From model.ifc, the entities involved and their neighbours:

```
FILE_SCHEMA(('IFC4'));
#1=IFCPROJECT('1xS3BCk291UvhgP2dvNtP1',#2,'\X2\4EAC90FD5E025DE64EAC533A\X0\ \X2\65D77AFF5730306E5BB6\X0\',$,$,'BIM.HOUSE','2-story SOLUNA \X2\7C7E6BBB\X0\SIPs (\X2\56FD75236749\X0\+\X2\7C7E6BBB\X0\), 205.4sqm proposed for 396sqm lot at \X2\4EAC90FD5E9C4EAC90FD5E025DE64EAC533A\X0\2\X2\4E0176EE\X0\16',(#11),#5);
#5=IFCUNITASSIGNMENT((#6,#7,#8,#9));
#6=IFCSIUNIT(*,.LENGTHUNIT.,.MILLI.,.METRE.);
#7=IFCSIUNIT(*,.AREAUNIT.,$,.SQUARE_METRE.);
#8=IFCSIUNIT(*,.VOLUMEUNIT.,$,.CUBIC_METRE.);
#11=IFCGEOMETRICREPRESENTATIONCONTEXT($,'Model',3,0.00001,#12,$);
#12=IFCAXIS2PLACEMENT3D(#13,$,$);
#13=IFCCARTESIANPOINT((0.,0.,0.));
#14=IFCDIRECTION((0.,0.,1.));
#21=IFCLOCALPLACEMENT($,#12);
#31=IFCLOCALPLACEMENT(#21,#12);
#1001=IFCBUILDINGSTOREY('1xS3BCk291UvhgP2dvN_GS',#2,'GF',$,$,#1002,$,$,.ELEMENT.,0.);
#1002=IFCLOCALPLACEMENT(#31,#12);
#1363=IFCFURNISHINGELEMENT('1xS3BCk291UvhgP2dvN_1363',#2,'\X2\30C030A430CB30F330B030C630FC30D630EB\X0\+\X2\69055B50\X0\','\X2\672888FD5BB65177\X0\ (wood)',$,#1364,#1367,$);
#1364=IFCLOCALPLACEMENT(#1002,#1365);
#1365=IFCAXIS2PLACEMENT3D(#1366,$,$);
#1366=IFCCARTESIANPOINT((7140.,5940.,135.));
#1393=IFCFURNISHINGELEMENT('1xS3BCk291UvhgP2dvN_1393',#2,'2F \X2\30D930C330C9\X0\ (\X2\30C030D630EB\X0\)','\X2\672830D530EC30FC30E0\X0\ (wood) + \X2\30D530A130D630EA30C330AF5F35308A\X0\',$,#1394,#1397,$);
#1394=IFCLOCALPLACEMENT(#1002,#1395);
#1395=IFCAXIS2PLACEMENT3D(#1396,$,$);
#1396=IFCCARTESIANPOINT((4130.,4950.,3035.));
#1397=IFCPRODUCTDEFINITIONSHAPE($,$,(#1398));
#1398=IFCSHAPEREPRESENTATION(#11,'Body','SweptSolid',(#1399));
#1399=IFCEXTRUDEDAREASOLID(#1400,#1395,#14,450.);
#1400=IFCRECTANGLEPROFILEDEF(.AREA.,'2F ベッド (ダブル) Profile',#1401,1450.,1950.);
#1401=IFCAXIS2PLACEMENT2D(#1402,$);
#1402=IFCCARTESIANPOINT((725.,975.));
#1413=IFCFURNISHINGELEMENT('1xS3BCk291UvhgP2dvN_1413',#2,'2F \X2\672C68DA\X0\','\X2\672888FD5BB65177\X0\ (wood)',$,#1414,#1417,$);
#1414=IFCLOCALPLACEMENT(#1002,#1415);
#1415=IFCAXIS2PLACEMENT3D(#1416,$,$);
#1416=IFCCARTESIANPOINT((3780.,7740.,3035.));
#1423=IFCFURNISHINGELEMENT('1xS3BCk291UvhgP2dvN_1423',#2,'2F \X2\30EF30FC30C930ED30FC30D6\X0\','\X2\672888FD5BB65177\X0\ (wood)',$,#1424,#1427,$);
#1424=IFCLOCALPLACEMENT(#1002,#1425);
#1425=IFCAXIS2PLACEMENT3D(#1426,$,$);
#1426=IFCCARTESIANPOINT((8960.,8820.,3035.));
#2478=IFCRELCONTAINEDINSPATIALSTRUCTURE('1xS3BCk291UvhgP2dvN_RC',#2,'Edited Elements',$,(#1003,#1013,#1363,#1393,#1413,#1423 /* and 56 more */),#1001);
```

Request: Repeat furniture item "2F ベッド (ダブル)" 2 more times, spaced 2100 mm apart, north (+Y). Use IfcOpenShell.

```python
import numpy as np
import ifcopenshell
import ifcopenshell.api.geometry
import ifcopenshell.api.root
import ifcopenshell.util.element
import ifcopenshell.util.placement

model = ifcopenshell.open("model.ifc")


def reuse_history(source, copy):
    """copy_class also copies each property set's owner history, people and application; keep the originals."""
    for rel in copy.IsDefinedBy:
        if rel.is_a("IfcRelDefinesByProperties") and (history := rel.RelatingPropertyDefinition.OwnerHistory):
            rel.RelatingPropertyDefinition.OwnerHistory = source.OwnerHistory
            ifcopenshell.util.element.remove_deep2(model, history)


source = model.by_id(1393)
base = ifcopenshell.util.placement.get_local_placement(source.ObjectPlacement)
step = np.array([0.0, 1.0, 0.0]) * 2100.0

for i in range(1, 3):
    copy = ifcopenshell.api.root.copy_class(model, product=source)
    copy.Representation = ifcopenshell.util.element.copy_deep(
        model, source.Representation, exclude=["IfcGeometricRepresentationContext", "IfcRepresentationMap"]
    )
    reuse_history(source, copy)
    matrix = base.copy()
    matrix[:3, 3] += i * step
    print("added at", matrix[:3, 3].round(3) + 0.0)
    ifcopenshell.api.geometry.edit_object_placement(model, product=copy, matrix=matrix, is_si=False)

model.write("model_updated.ifc")
```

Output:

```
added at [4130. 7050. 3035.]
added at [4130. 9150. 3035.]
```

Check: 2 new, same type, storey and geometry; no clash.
